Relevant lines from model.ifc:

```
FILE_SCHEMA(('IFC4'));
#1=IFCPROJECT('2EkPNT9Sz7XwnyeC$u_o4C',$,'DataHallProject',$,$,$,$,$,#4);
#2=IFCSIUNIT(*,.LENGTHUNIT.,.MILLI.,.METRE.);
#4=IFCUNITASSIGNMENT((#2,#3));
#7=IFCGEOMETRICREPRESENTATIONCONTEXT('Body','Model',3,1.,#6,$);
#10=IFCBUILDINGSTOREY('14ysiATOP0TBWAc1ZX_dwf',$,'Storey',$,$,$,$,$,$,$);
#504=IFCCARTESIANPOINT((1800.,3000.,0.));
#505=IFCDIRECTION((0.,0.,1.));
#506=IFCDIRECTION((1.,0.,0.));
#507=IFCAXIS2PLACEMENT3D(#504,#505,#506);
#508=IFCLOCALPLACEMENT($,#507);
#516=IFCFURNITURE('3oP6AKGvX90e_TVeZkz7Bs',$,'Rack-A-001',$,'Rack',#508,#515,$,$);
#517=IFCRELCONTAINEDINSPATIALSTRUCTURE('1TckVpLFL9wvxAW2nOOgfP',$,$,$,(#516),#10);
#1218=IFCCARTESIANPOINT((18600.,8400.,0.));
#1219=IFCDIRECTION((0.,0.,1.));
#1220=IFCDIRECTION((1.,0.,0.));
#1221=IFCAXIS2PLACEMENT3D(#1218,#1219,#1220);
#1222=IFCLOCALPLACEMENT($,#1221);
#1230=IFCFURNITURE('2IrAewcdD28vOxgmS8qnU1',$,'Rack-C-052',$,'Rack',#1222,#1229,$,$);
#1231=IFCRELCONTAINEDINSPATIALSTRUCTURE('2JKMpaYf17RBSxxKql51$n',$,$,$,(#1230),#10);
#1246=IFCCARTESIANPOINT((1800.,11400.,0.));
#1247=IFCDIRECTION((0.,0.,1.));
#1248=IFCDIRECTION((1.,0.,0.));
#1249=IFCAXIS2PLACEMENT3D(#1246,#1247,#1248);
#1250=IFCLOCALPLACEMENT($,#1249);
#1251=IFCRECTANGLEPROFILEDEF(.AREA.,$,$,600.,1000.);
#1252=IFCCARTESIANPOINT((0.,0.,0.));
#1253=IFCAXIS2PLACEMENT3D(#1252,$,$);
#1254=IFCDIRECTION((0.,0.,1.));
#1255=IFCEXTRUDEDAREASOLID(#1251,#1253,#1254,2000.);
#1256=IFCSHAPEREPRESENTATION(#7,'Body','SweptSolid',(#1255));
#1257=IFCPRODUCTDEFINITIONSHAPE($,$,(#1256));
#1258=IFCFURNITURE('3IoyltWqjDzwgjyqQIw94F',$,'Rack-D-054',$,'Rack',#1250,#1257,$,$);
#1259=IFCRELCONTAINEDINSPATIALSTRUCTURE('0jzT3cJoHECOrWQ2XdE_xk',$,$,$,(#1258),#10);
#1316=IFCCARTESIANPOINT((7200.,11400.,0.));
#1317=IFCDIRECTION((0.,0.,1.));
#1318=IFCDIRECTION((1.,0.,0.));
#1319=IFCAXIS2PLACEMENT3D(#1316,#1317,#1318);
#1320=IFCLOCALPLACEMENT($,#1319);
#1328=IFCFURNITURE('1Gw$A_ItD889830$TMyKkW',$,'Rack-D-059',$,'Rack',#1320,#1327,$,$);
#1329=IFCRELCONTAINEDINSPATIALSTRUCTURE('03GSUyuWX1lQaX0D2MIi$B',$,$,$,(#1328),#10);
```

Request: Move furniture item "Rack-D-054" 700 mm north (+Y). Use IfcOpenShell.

```python
import ifcopenshell
import ifcopenshell.api.geometry
import ifcopenshell.util.placement
import ifcopenshell.util.unit

model = ifcopenshell.open("model.ifc")
unit_scale = ifcopenshell.util.unit.calculate_unit_scale(model)

item = model.by_guid("3IoyltWqjDzwgjyqQIw94F")
matrix = ifcopenshell.util.placement.get_local_placement(item.ObjectPlacement)
matrix[1, 3] += 0.7 / unit_scale
ifcopenshell.api.geometry.edit_object_placement(model, product=item, matrix=matrix, is_si=False)

print(ifcopenshell.util.placement.get_local_placement(item.ObjectPlacement).round(3) + 0.0)

model.write("model_v2.ifc")
```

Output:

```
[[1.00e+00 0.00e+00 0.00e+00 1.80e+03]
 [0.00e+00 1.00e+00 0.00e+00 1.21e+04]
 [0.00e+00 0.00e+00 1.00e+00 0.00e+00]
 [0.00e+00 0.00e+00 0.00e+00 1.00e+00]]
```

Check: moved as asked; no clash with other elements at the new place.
